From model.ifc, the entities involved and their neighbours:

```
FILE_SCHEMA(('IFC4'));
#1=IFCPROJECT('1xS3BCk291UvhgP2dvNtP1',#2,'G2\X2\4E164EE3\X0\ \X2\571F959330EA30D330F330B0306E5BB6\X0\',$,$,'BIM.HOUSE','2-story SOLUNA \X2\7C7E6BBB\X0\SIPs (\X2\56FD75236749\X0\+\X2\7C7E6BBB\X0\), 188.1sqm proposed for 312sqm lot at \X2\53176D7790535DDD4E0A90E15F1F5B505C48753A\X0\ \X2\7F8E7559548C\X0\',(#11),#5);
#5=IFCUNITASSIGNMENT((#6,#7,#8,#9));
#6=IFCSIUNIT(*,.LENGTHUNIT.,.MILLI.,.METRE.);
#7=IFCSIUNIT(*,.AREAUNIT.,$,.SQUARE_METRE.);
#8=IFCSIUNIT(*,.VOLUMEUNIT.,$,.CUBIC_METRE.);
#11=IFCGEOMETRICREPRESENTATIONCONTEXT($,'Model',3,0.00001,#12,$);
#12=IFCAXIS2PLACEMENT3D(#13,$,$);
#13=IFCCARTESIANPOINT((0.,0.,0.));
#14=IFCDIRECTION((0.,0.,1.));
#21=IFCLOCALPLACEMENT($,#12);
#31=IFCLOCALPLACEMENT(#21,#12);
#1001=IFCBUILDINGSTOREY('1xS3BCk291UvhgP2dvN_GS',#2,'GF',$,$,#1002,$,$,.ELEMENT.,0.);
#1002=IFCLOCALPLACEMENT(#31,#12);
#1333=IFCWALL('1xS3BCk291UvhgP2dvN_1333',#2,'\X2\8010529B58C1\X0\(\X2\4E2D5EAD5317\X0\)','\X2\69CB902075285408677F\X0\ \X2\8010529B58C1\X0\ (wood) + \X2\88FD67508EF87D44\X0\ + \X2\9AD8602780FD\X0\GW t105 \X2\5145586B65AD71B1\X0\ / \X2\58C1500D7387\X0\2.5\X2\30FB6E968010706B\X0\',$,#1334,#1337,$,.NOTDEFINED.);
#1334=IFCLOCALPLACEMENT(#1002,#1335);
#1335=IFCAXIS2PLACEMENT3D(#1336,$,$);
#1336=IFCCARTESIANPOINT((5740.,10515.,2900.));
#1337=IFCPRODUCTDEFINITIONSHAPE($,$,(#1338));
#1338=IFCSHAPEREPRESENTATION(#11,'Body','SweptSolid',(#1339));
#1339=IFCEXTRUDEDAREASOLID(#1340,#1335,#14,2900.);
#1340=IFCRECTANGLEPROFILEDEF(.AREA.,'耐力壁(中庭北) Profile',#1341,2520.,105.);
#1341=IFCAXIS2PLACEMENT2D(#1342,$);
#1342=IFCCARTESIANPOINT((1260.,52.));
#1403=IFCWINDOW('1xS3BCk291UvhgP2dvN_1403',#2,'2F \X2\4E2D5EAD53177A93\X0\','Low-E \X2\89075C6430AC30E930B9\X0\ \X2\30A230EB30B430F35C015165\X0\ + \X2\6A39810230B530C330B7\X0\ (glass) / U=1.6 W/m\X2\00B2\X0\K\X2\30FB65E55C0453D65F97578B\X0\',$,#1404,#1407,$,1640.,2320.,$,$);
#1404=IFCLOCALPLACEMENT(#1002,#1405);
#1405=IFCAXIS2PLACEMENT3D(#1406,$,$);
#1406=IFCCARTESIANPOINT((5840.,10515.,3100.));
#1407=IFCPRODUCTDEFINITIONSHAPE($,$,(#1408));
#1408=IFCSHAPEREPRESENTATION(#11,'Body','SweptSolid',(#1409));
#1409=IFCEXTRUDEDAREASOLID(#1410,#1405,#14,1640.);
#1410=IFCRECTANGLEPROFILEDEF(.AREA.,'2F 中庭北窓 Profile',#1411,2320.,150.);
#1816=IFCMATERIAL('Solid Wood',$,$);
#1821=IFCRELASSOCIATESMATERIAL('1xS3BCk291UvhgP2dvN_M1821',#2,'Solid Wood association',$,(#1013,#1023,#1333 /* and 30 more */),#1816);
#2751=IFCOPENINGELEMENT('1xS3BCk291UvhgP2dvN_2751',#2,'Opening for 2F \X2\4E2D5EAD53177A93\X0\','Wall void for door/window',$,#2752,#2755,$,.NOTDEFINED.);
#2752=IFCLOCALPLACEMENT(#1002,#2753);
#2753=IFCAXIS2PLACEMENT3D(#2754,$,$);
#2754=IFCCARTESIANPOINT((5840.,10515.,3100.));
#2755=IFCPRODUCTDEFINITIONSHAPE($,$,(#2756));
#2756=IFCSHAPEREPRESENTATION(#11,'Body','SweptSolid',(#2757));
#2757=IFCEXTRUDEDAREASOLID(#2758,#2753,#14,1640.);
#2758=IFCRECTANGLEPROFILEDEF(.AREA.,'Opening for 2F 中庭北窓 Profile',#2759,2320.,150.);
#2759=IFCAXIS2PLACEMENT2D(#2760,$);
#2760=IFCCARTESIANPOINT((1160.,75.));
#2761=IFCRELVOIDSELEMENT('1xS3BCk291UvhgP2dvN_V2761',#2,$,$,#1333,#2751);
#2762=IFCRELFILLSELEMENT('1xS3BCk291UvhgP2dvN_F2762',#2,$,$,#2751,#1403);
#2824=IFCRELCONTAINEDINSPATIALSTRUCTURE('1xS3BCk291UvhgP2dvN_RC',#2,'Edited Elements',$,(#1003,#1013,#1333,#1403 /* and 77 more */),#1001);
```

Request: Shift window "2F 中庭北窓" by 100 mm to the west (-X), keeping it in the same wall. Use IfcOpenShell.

```python
import ifcopenshell
import ifcopenshell.api.geometry
import ifcopenshell.util.placement

model = ifcopenshell.open("model.ifc")

window = model.by_id(1403)
opening = window.FillsVoids[0].RelatingOpeningElement
wall = opening.VoidsElements[0].RelatingBuildingElement

wall_matrix = ifcopenshell.util.placement.get_local_placement(wall.ObjectPlacement)
shift = wall_matrix[:3, 0] * -100.0
before = ifcopenshell.util.placement.get_local_placement(window.ObjectPlacement)[:3, 3].copy()

# The window is not placed relative to its opening, so move both.
for product in (opening, window):
    matrix = ifcopenshell.util.placement.get_local_placement(product.ObjectPlacement)
    matrix[:3, 3] += shift
    ifcopenshell.api.geometry.edit_object_placement(model, product=product, matrix=matrix, is_si=False)

after = ifcopenshell.util.placement.get_local_placement(window.ObjectPlacement)[:3, 3]
print("window moved by", (after - before).round(3) + 0.0)

model.write("model_rev.ifc")
```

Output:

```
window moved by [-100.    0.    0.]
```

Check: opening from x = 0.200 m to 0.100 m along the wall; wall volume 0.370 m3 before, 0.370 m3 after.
